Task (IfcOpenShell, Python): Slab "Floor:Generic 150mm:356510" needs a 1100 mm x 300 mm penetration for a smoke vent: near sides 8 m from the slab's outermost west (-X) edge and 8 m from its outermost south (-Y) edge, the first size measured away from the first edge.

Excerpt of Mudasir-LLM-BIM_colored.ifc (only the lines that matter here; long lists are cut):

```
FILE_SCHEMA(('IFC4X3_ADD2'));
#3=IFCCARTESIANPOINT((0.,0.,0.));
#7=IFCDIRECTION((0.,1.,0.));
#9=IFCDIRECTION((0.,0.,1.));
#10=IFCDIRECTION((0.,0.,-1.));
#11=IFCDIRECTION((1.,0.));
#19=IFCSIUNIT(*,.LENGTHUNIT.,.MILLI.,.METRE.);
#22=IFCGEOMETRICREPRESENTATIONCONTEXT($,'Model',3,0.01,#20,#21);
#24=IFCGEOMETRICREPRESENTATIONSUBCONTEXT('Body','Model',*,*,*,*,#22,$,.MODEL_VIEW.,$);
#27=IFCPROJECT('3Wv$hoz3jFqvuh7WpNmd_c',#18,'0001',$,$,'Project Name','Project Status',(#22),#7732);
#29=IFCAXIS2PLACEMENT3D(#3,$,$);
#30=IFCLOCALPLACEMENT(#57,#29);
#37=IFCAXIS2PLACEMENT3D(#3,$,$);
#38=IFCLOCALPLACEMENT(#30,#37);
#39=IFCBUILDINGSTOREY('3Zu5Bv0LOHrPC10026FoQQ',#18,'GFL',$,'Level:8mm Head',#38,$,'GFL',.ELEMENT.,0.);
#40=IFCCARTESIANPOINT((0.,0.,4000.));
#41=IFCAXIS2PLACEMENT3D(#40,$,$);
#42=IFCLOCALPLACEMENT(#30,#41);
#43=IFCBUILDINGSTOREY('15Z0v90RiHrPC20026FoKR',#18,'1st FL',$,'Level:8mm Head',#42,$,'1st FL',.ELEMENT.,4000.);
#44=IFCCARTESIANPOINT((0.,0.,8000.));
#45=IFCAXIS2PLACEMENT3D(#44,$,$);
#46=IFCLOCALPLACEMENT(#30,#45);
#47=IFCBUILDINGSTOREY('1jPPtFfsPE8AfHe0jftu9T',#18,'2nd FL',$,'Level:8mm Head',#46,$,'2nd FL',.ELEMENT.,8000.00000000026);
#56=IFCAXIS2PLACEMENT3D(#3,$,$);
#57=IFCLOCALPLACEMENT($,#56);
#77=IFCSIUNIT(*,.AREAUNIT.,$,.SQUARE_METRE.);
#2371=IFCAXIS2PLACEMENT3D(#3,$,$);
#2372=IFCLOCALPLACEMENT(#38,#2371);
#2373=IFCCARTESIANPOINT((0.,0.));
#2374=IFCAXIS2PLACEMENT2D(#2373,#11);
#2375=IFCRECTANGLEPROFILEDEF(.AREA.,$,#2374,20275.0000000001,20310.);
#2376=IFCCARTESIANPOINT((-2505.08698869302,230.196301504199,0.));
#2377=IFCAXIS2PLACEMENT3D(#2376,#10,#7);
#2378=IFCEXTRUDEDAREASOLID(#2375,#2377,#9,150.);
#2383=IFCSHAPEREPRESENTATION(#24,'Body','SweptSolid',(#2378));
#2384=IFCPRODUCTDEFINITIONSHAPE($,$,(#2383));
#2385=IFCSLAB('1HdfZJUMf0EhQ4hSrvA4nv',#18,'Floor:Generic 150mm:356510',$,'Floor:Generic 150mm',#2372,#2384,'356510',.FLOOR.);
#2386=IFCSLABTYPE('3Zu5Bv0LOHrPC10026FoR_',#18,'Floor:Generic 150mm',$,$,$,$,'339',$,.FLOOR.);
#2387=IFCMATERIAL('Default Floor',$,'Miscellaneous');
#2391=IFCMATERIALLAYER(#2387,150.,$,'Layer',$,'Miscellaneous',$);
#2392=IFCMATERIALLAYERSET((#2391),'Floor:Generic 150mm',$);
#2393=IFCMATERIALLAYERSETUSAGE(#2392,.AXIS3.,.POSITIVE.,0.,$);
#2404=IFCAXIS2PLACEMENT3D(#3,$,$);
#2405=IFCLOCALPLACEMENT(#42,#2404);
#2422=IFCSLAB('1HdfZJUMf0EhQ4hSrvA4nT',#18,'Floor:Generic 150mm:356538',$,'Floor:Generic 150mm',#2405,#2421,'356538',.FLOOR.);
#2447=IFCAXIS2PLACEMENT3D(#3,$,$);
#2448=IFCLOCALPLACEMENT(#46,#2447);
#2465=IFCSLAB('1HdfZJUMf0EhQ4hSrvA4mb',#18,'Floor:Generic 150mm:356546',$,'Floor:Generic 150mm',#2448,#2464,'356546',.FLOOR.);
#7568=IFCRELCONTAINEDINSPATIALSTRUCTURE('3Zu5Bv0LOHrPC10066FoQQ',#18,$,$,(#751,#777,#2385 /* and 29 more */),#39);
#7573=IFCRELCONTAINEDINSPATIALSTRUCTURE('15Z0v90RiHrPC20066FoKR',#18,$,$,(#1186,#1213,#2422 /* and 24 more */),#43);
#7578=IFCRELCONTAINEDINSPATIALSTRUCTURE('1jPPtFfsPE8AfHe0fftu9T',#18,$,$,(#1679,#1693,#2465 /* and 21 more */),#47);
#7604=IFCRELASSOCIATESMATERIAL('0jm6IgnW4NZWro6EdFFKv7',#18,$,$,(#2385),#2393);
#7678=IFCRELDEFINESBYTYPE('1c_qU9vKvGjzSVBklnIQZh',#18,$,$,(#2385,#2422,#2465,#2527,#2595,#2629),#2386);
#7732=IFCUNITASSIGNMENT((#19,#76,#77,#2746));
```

```python
import numpy as np
import ifcopenshell
import ifcopenshell.api.feature
import ifcopenshell.api.geometry
import ifcopenshell.api.root
import ifcopenshell.geom
import ifcopenshell.util.placement
import ifcopenshell.util.representation
import ifcopenshell.util.shape
import ifcopenshell.util.unit

model = ifcopenshell.open("Mudasir-LLM-BIM_colored.ifc")
unit_scale = ifcopenshell.util.unit.calculate_unit_scale(model)
settings = ifcopenshell.geom.settings()


def volume(element):
    """Net volume in cubic metres, openings subtracted."""
    shape = ifcopenshell.geom.create_shape(settings, element)
    return ifcopenshell.util.shape.get_volume(shape.geometry)


slab = model.by_id(2385)
before = volume(slab)

# Extent in the slab's own axes, in metres. The edges named are its -X and -Y sides.
slab_shape = ifcopenshell.geom.create_shape(settings, slab)
vertices = ifcopenshell.util.shape.get_vertices(slab_shape.geometry)
x_min, y_min, bottom = vertices.min(axis=0)
top = vertices[:, 2].max()

opening = ifcopenshell.api.root.create_entity(model, ifc_class="IfcOpeningElement", name="Smoke vent opening", predefined_type="OPENING")
context = ifcopenshell.util.representation.get_context(model, "Model", "Body", "MODEL_VIEW")
width, depth = 1.1, 0.3
outline = [(0.0, 0.0), (width, 0.0), (width, depth), (0.0, depth), (0.0, 0.0)]
# Overshoot both faces by 50 mm so the cut is clean.
shape = ifcopenshell.api.geometry.add_slab_representation(
    model, context=context, depth=top - bottom + 0.1, polyline=outline
)
ifcopenshell.api.geometry.assign_representation(model, product=opening, representation=shape)

matrix = ifcopenshell.util.placement.get_local_placement(slab.ObjectPlacement)
matrix[:, 3] = matrix @ np.append(np.array([x_min + 8, y_min + 8, bottom - 0.05]) / unit_scale, 1.0)
ifcopenshell.api.geometry.edit_object_placement(model, product=opening, matrix=matrix, is_si=False)
ifcopenshell.api.feature.add_feature(model, feature=opening, element=slab)

after = volume(slab)

print(f"slab volume {before:.3f} -> {after:.3f} m3")

model.write("Mudasir-LLM-BIM_colored_edited.ifc")
```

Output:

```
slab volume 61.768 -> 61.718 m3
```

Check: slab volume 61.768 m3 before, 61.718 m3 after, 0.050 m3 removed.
